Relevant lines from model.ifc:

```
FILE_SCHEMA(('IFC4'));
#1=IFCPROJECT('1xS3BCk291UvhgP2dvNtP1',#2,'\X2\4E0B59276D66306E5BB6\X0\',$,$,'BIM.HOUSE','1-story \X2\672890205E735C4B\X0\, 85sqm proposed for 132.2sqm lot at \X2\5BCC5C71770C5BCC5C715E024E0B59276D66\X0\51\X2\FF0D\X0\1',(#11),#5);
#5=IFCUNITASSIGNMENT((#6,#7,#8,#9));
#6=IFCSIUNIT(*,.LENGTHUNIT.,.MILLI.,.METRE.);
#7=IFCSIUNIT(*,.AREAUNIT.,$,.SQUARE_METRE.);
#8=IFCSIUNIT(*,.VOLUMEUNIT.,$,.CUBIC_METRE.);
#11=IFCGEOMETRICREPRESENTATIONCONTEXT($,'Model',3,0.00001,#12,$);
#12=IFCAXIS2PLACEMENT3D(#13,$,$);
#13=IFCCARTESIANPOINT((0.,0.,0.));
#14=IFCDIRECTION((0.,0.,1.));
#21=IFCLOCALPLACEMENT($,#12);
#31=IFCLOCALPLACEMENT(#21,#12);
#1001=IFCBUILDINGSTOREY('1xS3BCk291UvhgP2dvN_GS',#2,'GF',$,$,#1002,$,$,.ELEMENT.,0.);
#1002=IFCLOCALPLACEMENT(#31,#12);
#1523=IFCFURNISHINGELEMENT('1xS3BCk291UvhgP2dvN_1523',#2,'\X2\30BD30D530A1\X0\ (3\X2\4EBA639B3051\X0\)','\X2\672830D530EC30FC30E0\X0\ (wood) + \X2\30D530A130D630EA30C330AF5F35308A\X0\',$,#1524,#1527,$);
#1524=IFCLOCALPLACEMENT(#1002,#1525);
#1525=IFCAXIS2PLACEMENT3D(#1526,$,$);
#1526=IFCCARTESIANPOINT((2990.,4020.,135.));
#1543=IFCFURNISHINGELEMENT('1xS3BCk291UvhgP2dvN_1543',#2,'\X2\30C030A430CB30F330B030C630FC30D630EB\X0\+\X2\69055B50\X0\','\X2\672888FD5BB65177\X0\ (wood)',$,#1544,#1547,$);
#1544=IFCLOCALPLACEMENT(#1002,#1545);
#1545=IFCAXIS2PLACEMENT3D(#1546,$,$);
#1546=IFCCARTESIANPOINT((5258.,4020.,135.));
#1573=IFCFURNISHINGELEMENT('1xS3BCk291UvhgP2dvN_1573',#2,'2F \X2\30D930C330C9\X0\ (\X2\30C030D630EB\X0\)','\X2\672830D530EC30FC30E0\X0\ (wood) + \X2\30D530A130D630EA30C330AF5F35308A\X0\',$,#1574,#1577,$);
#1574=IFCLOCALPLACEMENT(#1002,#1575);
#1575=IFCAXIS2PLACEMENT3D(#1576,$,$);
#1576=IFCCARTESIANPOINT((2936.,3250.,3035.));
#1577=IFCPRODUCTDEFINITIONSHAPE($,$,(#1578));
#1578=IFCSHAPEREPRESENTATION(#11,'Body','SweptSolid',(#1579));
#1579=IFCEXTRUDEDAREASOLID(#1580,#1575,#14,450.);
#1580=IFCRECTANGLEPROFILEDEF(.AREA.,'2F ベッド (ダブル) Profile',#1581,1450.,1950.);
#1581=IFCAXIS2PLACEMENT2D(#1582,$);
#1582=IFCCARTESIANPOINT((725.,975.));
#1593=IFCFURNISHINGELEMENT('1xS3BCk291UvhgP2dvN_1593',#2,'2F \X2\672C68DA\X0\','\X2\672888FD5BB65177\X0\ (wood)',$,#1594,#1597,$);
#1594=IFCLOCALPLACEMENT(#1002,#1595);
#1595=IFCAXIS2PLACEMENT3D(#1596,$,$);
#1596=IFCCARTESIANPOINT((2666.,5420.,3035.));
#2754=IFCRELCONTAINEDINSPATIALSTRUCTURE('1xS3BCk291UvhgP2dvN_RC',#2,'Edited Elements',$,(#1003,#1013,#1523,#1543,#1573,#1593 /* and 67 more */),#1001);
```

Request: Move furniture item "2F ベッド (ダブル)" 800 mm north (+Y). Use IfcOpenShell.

```python
import ifcopenshell
import ifcopenshell.api.geometry
import ifcopenshell.util.placement
import ifcopenshell.util.unit

model = ifcopenshell.open("model.ifc")
unit_scale = ifcopenshell.util.unit.calculate_unit_scale(model)

item = model.by_guid("1xS3BCk291UvhgP2dvN_1573")
matrix = ifcopenshell.util.placement.get_local_placement(item.ObjectPlacement)
matrix[1, 3] += 0.8 / unit_scale
ifcopenshell.api.geometry.edit_object_placement(model, product=item, matrix=matrix, is_si=False)

print(ifcopenshell.util.placement.get_local_placement(item.ObjectPlacement).round(3) + 0.0)

model.write("model_v2.ifc")
```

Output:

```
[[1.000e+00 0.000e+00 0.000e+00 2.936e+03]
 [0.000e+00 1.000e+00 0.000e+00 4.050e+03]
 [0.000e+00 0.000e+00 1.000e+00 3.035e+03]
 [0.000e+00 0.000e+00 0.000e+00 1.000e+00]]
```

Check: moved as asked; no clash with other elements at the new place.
